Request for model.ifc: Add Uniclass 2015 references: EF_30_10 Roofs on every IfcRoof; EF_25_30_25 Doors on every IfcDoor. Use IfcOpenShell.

First a look at what the model holds.

```python
import ifcopenshell

model = ifcopenshell.open("model.ifc")
print(model.schema)
print("classifications:", [c.Name for c in model.by_type("IfcClassification")])
for ifc_class in ("IfcDoor", "IfcRoof", "IfcStair", "IfcWall", "IfcWindow"):
    print(ifc_class, len(model.by_type(ifc_class)))
```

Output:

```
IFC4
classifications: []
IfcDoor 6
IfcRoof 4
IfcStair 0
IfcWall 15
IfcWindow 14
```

```python
import ifcopenshell
import ifcopenshell.api.classification

model = ifcopenshell.open("model.ifc")

system = ifcopenshell.api.classification.add_classification(model, classification="Uniclass 2015")

codes = {
    "IfcRoof": ("EF_30_10", "Roofs"),
    "IfcDoor": ("EF_25_30_25", "Doors"),
}
for ifc_class, (code, name) in codes.items():
    products = model.by_type(ifc_class)
    ifcopenshell.api.classification.add_reference(
        model, products=products, classification=system, identification=code, name=name
    )
    print(code, len(products))

model.write("model_rev.ifc")
```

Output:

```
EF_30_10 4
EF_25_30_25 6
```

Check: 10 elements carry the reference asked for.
